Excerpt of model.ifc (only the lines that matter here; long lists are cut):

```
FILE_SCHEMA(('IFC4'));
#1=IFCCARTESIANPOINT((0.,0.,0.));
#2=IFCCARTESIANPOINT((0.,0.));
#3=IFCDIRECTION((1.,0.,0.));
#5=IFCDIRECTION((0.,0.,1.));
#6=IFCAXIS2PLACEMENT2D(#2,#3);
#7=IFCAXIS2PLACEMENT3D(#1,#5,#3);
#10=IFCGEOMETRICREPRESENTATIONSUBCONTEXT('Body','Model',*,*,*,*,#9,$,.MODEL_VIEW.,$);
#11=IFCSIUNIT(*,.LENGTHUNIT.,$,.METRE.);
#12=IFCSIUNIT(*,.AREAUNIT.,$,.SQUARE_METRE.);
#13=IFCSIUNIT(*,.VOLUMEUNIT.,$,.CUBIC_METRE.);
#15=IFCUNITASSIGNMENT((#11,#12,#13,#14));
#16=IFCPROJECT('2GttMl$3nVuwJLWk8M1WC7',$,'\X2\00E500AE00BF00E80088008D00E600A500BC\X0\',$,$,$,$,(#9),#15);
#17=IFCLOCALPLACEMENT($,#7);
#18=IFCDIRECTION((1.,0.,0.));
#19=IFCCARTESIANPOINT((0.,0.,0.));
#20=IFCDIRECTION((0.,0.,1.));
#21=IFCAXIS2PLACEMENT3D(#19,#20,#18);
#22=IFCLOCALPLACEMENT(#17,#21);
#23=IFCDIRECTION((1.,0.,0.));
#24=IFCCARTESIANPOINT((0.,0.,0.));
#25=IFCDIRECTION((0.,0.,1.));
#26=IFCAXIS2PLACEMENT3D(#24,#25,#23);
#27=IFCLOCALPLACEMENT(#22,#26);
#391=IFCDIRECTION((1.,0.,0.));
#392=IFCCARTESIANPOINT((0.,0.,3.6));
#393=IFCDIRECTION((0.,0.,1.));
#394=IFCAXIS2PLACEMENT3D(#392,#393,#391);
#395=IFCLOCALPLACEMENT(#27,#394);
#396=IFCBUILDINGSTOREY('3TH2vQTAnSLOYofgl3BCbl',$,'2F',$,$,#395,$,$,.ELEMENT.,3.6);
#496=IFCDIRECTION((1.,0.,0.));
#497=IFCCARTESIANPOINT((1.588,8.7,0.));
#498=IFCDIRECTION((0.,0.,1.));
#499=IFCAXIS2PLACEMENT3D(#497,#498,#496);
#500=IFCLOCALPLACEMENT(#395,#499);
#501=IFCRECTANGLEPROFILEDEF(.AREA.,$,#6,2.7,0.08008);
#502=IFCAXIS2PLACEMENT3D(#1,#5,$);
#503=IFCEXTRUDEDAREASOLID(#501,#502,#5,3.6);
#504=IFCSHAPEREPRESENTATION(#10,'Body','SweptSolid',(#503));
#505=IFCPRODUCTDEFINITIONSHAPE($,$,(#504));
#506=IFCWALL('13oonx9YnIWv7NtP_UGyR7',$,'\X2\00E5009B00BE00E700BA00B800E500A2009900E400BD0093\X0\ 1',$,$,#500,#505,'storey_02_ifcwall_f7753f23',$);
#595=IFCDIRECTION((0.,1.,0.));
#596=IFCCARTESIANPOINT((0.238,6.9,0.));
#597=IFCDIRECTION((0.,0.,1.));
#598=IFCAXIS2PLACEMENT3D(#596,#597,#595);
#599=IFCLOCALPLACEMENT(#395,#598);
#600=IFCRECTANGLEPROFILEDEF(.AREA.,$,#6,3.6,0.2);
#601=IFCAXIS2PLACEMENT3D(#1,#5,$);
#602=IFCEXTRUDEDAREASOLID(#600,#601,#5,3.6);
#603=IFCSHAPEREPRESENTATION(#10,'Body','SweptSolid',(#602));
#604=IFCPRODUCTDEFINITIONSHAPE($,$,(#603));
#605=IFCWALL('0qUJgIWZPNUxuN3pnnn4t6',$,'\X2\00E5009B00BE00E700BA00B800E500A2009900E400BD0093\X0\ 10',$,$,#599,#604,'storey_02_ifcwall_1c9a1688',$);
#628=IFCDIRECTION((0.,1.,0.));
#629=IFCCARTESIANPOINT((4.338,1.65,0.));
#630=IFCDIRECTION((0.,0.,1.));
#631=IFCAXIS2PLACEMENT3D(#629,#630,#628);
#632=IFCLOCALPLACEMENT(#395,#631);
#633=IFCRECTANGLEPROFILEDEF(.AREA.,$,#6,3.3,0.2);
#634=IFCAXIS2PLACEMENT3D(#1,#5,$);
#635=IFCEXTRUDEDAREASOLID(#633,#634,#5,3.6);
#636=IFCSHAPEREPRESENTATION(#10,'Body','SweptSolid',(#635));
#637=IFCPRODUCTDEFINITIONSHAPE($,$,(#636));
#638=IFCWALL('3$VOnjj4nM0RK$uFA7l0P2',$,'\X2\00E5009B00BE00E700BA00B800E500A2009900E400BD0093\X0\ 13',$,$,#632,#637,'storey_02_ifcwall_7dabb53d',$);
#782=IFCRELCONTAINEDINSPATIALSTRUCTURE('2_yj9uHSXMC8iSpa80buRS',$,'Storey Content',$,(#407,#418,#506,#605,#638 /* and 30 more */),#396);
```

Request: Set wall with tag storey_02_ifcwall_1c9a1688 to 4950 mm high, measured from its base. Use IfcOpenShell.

```python
import ifcopenshell
import ifcopenshell.geom
import ifcopenshell.util.representation
import ifcopenshell.util.shape

model = ifcopenshell.open("model.ifc")
settings = ifcopenshell.geom.settings()


def volume(element):
    """Net volume in cubic metres, openings subtracted."""
    shape = ifcopenshell.geom.create_shape(settings, element)
    return ifcopenshell.util.shape.get_volume(shape.geometry)


wall = model.by_id(605)
before = volume(wall)

body = ifcopenshell.util.representation.get_representation(wall, "Model", "Body")
solid = body.Items[0]
old_height = solid.Depth
solid.Depth = 4.95
after = volume(wall)

print(f"height {old_height:g} -> {solid.Depth:g}, volume {before:.3f} -> {after:.3f} m3")

model.write("model_updated.ifc")
```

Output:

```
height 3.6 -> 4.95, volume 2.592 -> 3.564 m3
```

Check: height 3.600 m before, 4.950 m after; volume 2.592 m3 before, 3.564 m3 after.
